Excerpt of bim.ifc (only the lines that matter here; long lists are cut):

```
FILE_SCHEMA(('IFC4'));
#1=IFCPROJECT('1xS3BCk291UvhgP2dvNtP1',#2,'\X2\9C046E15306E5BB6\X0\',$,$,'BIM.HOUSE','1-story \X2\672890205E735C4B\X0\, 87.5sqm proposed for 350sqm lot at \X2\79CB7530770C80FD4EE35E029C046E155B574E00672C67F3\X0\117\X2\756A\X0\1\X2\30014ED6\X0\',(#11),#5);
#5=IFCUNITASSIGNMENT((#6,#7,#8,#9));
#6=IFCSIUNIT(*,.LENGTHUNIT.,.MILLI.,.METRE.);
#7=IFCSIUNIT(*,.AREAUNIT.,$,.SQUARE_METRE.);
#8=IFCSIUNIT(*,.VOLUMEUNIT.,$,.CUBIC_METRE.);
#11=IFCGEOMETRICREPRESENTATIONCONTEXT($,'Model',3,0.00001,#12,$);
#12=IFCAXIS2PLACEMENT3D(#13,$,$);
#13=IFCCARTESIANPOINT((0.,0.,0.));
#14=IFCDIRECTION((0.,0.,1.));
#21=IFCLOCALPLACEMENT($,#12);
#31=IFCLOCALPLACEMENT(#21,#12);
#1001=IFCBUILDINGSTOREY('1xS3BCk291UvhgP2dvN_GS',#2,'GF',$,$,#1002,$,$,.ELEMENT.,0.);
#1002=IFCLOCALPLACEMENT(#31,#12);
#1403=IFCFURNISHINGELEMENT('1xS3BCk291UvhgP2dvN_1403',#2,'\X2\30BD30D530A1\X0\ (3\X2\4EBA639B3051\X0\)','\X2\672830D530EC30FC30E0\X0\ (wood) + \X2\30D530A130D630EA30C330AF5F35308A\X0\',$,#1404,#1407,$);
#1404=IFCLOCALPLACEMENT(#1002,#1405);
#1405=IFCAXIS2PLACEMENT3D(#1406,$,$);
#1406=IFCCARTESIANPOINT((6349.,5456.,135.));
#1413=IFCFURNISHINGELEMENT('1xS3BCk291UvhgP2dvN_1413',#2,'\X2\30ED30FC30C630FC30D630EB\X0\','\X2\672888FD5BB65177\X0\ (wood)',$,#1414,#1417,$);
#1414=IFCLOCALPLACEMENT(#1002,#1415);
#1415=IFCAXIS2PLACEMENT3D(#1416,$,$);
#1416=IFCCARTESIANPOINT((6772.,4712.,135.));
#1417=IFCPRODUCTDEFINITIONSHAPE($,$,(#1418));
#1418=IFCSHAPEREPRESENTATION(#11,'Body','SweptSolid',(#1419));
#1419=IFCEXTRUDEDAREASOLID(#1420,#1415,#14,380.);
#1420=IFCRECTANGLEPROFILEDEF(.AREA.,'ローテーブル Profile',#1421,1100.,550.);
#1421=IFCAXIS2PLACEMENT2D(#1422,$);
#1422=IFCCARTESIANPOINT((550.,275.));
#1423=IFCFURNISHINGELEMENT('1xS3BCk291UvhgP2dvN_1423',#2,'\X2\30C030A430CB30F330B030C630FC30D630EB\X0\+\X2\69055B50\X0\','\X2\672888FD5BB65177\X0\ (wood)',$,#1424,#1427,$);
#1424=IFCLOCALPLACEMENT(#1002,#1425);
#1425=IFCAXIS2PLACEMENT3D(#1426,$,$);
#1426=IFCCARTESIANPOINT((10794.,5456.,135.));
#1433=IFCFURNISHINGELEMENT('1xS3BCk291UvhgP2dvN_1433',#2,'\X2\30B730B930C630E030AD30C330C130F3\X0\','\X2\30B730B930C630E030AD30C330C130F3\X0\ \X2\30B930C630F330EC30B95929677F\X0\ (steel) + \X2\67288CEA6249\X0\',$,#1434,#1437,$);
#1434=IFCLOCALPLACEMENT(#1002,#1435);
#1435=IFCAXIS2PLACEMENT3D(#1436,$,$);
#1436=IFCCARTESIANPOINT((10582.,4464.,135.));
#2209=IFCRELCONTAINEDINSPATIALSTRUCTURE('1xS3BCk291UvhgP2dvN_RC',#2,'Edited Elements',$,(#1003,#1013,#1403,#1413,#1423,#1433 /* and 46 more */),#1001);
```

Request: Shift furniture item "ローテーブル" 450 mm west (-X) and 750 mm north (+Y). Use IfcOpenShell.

```python
import ifcopenshell
import ifcopenshell.api.geometry
import ifcopenshell.util.placement
import ifcopenshell.util.unit

model = ifcopenshell.open("bim.ifc")
unit_scale = ifcopenshell.util.unit.calculate_unit_scale(model)

item = model.by_guid("1xS3BCk291UvhgP2dvN_1413")
matrix = ifcopenshell.util.placement.get_local_placement(item.ObjectPlacement)
matrix[0, 3] -= 0.45 / unit_scale
matrix[1, 3] += 0.75 / unit_scale
ifcopenshell.api.geometry.edit_object_placement(model, product=item, matrix=matrix, is_si=False)

print(ifcopenshell.util.placement.get_local_placement(item.ObjectPlacement).round(3) + 0.0)

model.write("bim_rev.ifc")
```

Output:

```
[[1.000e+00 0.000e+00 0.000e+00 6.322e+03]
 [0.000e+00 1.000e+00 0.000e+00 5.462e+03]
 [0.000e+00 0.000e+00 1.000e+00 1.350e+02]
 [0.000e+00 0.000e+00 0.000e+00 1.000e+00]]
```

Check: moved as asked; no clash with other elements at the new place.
